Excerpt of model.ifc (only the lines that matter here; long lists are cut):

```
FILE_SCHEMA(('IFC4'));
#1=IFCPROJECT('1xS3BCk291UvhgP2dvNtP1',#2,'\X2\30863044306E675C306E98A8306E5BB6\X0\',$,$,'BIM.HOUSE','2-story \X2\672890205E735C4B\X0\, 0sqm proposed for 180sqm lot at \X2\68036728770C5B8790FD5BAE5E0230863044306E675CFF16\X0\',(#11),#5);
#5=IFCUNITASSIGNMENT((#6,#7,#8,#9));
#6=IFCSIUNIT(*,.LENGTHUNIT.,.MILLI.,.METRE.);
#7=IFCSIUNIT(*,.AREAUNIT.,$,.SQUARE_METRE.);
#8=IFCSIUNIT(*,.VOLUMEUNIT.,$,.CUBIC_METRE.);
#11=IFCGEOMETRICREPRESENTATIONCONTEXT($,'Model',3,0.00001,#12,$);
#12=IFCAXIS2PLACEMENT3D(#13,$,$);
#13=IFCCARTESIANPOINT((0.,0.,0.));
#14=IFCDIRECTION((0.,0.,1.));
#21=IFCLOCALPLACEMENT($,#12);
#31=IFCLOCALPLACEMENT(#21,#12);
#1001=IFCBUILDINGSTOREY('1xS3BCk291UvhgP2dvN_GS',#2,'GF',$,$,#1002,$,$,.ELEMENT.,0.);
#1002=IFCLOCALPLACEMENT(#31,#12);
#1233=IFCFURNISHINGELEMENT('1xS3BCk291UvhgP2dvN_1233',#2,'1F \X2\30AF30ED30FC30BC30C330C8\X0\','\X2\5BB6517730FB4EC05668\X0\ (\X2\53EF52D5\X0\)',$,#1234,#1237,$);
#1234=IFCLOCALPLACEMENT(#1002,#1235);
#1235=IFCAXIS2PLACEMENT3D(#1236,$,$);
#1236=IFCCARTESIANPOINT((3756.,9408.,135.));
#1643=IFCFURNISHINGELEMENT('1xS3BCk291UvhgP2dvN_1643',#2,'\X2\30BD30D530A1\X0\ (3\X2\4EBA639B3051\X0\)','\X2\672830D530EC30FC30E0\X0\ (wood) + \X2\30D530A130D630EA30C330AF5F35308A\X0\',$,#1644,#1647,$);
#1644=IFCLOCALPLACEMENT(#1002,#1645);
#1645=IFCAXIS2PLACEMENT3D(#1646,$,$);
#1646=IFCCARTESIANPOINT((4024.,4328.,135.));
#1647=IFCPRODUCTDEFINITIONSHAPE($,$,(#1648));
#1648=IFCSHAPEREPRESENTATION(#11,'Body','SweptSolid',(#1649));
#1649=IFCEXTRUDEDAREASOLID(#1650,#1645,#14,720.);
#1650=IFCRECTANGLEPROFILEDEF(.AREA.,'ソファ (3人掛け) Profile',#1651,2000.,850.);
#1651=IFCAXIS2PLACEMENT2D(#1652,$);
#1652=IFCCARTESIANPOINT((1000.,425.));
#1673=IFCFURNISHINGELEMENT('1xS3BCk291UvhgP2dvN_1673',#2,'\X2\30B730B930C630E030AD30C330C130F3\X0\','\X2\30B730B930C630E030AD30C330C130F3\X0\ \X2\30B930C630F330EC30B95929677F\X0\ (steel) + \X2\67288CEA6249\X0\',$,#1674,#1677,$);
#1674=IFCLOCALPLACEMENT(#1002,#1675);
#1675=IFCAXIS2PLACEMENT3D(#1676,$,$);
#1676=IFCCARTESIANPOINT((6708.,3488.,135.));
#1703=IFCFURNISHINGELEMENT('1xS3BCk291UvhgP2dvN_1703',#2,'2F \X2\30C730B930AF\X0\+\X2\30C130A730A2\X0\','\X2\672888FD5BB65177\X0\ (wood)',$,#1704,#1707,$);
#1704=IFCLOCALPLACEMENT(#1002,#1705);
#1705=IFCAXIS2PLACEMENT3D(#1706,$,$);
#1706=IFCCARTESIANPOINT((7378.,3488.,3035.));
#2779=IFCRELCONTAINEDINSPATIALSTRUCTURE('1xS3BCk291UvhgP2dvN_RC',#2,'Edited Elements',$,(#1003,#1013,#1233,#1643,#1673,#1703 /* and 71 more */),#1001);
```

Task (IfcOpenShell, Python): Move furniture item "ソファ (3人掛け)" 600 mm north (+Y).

```python
import ifcopenshell
import ifcopenshell.api.geometry
import ifcopenshell.util.placement

model = ifcopenshell.open("model.ifc")

item = model.by_id(1643)
matrix = ifcopenshell.util.placement.get_local_placement(item.ObjectPlacement)
matrix[1, 3] += 600.0
ifcopenshell.api.geometry.edit_object_placement(model, product=item, matrix=matrix, is_si=False)

print(ifcopenshell.util.placement.get_local_placement(item.ObjectPlacement).round(3) + 0.0)

model.write("model_rev.ifc")
```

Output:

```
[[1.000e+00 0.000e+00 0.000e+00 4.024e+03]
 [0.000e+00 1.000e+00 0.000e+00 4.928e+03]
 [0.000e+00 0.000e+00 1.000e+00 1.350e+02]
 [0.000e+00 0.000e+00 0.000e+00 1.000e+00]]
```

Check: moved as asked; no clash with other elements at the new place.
